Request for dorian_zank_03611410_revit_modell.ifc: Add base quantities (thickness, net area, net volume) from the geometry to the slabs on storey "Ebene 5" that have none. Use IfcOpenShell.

First a look at what the model holds.

```python
import ifcopenshell
import ifcopenshell.util.element
import ifcopenshell.util.unit

model = ifcopenshell.open("dorian_zank_03611410_revit_modell.ifc")
print(model.schema)
for unit_type in ("LENGTHUNIT", "AREAUNIT", "VOLUMEUNIT"):
    print(unit_type, ifcopenshell.util.unit.calculate_unit_scale(model, unit_type))
storey = next(s for s in model.by_type("IfcBuildingStorey") if s.Name == "Ebene 5")
slabs = [e for e in ifcopenshell.util.element.get_decomposition(storey) if e.is_a("IfcSlab")]
for e in sorted(slabs, key=lambda e: e.id()):
    print(e.id(), e.is_a(), e.Name, list(ifcopenshell.util.element.get_psets(e, qtos_only=True)), sep=" | ")
```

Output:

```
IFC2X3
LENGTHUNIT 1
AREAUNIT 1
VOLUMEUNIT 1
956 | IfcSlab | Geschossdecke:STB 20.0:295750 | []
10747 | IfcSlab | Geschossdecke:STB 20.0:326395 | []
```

```python
import ifcopenshell
import ifcopenshell.api.pset
import ifcopenshell.geom
import ifcopenshell.util.element
import ifcopenshell.util.shape
import ifcopenshell.util.unit

model = ifcopenshell.open("dorian_zank_03611410_revit_modell.ifc")
unit_scale = ifcopenshell.util.unit.calculate_unit_scale(model)
area_scale = ifcopenshell.util.unit.calculate_unit_scale(model, "AREAUNIT")
volume_scale = ifcopenshell.util.unit.calculate_unit_scale(model, "VOLUMEUNIT")
settings = ifcopenshell.geom.settings()

storey = next(s for s in model.by_type("IfcBuildingStorey") if s.Name == "Ebene 5")
slabs = [e for e in ifcopenshell.util.element.get_decomposition(storey) if e.is_a("IfcSlab")]

for e in sorted(slabs, key=lambda e: e.id()):
    if ifcopenshell.util.element.get_psets(e, qtos_only=True, should_inherit=False):
        continue
    # Geometry comes back in metres, in the element's own axes.
    shape = ifcopenshell.geom.create_shape(settings, e)
    values = {
        "Width": ifcopenshell.util.shape.get_z(shape.geometry) / unit_scale,
        "NetArea": ifcopenshell.util.shape.get_footprint_area(shape.geometry) / area_scale,
        "NetVolume": ifcopenshell.util.shape.get_volume(shape.geometry) / volume_scale,
    }
    qto = ifcopenshell.api.pset.add_qto(model, product=e, name="BaseQuantities")
    ifcopenshell.api.pset.edit_qto(model, qto=qto, properties=values)
    print(e.id(), {k: round(v, 3) for k, v in values.items()})

model.write("dorian_zank_03611410_revit_modell_v2.ifc")
```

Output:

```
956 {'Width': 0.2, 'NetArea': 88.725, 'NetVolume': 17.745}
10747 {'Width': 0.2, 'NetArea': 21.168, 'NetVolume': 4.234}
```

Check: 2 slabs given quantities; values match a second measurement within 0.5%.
